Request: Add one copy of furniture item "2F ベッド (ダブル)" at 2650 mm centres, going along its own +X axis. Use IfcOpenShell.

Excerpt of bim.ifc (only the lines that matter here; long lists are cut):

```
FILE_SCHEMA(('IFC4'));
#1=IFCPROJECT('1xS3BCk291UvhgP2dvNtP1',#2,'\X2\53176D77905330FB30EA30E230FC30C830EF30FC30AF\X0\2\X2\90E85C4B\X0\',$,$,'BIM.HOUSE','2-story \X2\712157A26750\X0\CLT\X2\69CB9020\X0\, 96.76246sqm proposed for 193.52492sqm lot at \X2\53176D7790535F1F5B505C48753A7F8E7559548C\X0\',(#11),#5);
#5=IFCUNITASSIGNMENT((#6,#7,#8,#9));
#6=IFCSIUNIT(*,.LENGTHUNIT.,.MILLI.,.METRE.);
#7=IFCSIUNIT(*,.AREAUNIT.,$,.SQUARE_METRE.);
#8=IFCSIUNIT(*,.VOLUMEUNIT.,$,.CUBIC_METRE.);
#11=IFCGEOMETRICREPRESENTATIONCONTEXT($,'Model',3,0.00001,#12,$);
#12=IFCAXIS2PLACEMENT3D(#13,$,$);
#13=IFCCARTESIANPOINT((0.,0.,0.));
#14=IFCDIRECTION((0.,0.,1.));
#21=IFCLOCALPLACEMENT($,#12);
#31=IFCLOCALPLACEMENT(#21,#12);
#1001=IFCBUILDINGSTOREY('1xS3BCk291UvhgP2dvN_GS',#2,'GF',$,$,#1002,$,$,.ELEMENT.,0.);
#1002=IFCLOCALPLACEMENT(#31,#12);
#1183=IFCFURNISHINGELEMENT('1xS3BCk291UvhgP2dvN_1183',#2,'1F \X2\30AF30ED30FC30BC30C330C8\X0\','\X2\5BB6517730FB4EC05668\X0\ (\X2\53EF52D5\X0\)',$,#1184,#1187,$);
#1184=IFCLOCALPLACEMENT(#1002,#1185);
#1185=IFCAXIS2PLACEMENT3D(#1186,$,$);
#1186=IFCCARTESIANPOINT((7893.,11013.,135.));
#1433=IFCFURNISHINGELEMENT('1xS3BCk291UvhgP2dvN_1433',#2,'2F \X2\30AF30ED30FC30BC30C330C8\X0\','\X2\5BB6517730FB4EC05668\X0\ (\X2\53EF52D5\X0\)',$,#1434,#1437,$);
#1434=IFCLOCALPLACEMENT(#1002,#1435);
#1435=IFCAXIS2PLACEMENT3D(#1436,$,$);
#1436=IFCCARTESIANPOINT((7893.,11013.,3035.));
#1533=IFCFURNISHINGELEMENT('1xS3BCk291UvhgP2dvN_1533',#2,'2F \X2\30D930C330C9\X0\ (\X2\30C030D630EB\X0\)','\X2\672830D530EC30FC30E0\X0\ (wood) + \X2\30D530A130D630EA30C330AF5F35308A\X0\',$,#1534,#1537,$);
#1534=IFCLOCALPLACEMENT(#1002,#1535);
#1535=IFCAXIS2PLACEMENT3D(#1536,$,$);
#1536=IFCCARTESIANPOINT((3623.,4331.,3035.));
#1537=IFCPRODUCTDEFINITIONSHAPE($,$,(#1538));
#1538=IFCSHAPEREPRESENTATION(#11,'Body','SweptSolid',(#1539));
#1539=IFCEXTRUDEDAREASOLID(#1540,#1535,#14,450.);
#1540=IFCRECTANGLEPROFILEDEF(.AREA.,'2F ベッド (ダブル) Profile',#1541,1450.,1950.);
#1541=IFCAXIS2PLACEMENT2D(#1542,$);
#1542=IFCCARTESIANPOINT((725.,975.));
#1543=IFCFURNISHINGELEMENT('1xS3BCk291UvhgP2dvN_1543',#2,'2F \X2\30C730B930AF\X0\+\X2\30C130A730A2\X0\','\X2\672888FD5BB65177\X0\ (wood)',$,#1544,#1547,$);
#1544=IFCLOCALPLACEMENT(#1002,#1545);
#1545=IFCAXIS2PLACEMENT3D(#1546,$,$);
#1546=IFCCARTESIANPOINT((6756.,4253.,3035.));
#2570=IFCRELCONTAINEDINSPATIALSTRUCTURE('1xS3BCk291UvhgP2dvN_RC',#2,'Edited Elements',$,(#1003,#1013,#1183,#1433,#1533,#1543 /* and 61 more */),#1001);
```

```python
import ifcopenshell
import ifcopenshell.api.geometry
import ifcopenshell.api.root
import ifcopenshell.util.element
import ifcopenshell.util.placement
import ifcopenshell.util.unit

model = ifcopenshell.open("bim.ifc")
unit_scale = ifcopenshell.util.unit.calculate_unit_scale(model)


def reuse_history(source, copy):
    """copy_class also copies each property set's owner history, people and application; keep the originals."""
    for rel in copy.IsDefinedBy:
        if rel.is_a("IfcRelDefinesByProperties") and (history := rel.RelatingPropertyDefinition.OwnerHistory):
            rel.RelatingPropertyDefinition.OwnerHistory = source.OwnerHistory
            ifcopenshell.util.element.remove_deep2(model, history)


source = model.by_guid("1xS3BCk291UvhgP2dvN_1533")
base = ifcopenshell.util.placement.get_local_placement(source.ObjectPlacement)
step = base[:3, 0] * 2.65 / unit_scale

for i in range(1, 2):
    copy = ifcopenshell.api.root.copy_class(model, product=source)
    copy.Representation = ifcopenshell.util.element.copy_deep(
        model, source.Representation, exclude=["IfcGeometricRepresentationContext", "IfcRepresentationMap"]
    )
    reuse_history(source, copy)
    matrix = base.copy()
    matrix[:3, 3] += i * step
    print("added at", matrix[:3, 3].round(3) + 0.0)
    ifcopenshell.api.geometry.edit_object_placement(model, product=copy, matrix=matrix, is_si=False)

model.write("bim_rev.ifc")
```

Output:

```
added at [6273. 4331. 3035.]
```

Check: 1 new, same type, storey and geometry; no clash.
